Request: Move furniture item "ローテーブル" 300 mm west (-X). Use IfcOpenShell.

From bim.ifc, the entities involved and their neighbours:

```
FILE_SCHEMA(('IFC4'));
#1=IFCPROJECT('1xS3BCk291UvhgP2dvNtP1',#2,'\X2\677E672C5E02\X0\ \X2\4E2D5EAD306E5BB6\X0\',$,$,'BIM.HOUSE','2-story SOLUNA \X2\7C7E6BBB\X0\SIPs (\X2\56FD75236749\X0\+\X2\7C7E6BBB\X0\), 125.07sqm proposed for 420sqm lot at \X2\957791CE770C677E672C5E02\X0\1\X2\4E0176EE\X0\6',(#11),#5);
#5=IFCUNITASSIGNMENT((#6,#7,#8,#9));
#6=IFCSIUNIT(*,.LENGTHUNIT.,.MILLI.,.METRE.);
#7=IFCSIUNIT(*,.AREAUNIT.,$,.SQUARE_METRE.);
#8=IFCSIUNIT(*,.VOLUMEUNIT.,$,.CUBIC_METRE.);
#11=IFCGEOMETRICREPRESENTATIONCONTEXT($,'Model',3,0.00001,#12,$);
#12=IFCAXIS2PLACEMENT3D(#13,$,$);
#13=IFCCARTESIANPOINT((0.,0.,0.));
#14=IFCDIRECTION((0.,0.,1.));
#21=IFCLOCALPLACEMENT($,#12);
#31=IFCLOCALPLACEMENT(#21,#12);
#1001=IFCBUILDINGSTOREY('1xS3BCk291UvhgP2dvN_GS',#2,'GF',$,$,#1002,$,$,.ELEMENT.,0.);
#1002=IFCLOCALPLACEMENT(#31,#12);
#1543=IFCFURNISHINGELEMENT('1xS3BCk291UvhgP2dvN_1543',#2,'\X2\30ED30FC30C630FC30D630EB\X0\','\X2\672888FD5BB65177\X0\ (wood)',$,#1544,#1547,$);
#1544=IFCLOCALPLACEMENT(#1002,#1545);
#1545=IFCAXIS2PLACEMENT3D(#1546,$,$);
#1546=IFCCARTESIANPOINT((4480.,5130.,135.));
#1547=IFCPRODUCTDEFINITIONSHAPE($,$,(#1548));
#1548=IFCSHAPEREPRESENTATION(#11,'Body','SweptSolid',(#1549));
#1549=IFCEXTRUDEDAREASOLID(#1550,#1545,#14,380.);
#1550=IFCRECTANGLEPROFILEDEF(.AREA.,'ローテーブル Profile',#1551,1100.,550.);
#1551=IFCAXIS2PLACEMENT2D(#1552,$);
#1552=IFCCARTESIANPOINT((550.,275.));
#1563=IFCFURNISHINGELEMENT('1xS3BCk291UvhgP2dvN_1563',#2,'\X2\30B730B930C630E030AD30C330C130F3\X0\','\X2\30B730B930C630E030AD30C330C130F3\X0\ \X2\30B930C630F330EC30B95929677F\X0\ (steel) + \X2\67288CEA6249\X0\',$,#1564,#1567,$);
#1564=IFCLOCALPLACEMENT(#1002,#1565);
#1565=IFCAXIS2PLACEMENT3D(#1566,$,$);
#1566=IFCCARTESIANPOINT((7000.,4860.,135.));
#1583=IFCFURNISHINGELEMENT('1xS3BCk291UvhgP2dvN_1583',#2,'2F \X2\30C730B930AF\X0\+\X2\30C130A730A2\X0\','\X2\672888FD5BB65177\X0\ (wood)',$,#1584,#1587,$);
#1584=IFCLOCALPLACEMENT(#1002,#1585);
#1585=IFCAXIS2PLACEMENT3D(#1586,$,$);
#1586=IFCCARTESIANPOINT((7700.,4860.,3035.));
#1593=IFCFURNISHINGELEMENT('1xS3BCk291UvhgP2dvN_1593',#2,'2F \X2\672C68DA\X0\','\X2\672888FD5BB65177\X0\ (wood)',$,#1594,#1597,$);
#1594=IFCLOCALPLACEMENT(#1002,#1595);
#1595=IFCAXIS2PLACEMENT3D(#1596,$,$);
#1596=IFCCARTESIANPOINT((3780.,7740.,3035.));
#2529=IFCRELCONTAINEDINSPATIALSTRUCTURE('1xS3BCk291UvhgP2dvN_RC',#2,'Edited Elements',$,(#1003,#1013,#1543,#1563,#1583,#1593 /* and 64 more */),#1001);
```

```python
import ifcopenshell
import ifcopenshell.api.geometry
import ifcopenshell.util.placement
import ifcopenshell.util.unit

model = ifcopenshell.open("bim.ifc")
unit_scale = ifcopenshell.util.unit.calculate_unit_scale(model)

item = model.by_guid("1xS3BCk291UvhgP2dvN_1543")
matrix = ifcopenshell.util.placement.get_local_placement(item.ObjectPlacement)
matrix[0, 3] -= 0.3 / unit_scale
ifcopenshell.api.geometry.edit_object_placement(model, product=item, matrix=matrix, is_si=False)

print(ifcopenshell.util.placement.get_local_placement(item.ObjectPlacement).round(3) + 0.0)

model.write("bim-out.ifc")
```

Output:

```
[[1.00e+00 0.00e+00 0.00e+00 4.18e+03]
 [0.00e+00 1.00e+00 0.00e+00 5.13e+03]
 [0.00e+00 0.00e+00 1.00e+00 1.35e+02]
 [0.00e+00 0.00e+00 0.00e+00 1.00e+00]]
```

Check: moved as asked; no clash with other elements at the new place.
